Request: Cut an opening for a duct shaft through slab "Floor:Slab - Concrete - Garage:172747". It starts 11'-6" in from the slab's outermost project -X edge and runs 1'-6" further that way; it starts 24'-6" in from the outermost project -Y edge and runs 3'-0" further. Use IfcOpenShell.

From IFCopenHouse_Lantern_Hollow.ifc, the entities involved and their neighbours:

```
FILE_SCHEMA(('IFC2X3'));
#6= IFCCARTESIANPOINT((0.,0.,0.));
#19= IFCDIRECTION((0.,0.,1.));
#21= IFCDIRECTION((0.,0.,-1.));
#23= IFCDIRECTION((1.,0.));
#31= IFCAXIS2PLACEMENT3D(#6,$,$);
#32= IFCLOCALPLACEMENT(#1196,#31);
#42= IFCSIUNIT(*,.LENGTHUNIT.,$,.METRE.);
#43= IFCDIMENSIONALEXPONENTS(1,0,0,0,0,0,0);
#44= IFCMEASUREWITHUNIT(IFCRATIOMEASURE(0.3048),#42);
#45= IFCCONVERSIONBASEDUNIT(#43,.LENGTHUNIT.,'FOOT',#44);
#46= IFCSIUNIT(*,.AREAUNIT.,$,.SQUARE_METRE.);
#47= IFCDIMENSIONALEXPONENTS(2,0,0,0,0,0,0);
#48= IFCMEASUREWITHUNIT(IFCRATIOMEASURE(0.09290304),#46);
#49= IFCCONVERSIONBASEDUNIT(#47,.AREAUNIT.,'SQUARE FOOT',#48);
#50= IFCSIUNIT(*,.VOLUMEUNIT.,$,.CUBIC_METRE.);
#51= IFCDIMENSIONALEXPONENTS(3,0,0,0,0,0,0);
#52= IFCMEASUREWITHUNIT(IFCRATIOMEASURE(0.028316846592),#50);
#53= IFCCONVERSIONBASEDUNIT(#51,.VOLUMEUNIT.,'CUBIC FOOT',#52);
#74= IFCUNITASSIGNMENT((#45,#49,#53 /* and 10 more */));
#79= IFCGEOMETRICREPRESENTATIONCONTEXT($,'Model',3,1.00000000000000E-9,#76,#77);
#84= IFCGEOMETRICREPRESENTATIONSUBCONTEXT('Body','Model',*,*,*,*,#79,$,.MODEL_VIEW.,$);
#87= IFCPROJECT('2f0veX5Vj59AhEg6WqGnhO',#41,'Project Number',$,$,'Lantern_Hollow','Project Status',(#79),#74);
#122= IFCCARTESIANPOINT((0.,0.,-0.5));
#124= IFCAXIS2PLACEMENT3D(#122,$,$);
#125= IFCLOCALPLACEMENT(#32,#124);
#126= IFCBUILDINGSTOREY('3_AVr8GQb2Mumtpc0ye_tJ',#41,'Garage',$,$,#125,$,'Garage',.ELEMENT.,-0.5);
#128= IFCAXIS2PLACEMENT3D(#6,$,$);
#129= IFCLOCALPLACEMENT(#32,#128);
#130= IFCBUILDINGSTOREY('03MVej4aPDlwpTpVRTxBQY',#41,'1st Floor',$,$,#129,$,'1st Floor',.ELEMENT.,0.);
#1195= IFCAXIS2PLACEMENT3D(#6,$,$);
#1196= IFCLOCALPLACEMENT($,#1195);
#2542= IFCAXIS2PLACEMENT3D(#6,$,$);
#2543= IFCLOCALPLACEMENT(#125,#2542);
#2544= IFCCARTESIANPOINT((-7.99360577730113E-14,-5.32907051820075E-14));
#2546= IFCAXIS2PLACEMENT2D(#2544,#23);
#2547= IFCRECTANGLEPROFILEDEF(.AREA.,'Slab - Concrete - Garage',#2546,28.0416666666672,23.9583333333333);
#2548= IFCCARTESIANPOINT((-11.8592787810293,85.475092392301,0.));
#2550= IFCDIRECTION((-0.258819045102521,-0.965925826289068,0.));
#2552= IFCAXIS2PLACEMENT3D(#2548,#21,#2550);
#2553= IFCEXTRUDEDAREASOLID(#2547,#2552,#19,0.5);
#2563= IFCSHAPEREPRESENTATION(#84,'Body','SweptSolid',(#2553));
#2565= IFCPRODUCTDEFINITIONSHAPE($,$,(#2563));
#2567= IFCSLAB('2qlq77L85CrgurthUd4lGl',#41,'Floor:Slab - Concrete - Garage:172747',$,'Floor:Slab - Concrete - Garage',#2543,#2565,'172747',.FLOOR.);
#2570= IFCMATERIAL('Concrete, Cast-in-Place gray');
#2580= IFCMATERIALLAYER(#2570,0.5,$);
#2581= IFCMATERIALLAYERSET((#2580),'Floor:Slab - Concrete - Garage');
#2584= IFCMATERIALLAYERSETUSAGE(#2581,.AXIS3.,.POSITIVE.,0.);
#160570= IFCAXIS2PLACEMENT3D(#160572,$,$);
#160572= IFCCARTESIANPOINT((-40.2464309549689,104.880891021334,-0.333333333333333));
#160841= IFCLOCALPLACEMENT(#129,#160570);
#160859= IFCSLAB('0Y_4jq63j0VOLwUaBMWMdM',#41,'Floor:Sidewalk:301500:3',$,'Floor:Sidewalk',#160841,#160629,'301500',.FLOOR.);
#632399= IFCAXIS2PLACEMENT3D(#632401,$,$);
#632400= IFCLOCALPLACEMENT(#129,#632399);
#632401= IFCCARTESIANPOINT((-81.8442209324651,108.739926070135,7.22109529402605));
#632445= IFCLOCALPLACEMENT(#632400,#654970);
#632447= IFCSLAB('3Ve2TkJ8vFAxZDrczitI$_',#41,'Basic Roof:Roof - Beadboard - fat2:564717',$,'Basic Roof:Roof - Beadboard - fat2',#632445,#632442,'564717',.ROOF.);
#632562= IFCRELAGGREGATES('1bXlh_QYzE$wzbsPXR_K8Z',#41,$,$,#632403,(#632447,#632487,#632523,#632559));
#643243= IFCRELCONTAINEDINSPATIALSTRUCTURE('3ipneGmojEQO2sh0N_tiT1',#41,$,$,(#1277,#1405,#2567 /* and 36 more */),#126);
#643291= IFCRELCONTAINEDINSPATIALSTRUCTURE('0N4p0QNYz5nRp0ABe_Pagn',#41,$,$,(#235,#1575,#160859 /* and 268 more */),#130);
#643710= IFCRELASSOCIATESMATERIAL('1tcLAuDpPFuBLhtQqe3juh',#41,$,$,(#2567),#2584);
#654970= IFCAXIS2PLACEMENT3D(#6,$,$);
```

```python
import numpy as np
import ifcopenshell
import ifcopenshell.api.feature
import ifcopenshell.api.geometry
import ifcopenshell.api.root
import ifcopenshell.geom
import ifcopenshell.util.placement
import ifcopenshell.util.representation
import ifcopenshell.util.shape
import ifcopenshell.util.unit

model = ifcopenshell.open("IFCopenHouse_Lantern_Hollow.ifc")
unit_scale = ifcopenshell.util.unit.calculate_unit_scale(model)
settings = ifcopenshell.geom.settings()


def volume(element):
    """Net volume in cubic metres, openings subtracted."""
    shape = ifcopenshell.geom.create_shape(settings, element)
    return ifcopenshell.util.shape.get_volume(shape.geometry)


slab = model.by_id(2567)
before = volume(slab)

# Extent in the slab's own axes, in metres. The edges named are its -X and -Y sides.
slab_shape = ifcopenshell.geom.create_shape(settings, slab)
vertices = ifcopenshell.util.shape.get_vertices(slab_shape.geometry)
x_min, y_min, bottom = vertices.min(axis=0)
top = vertices[:, 2].max()

opening = ifcopenshell.api.root.create_entity(model, ifc_class="IfcOpeningElement", name="Duct shaft opening")
context = ifcopenshell.util.representation.get_context(model, "Model", "Body", "MODEL_VIEW")
width, depth = 0.4572, 0.9144
outline = [(0.0, 0.0), (width, 0.0), (width, depth), (0.0, depth), (0.0, 0.0)]
# Overshoot both faces by 50 mm so the cut is clean.
shape = ifcopenshell.api.geometry.add_slab_representation(
    model, context=context, depth=top - bottom + 0.1, polyline=outline
)
ifcopenshell.api.geometry.assign_representation(model, product=opening, representation=shape)

matrix = ifcopenshell.util.placement.get_local_placement(slab.ObjectPlacement)
matrix[:, 3] = matrix @ np.append(np.array([x_min + 3.5052, y_min + 7.4676, bottom - 0.05]) / unit_scale, 1.0)
ifcopenshell.api.geometry.edit_object_placement(model, product=opening, matrix=matrix, is_si=False)
ifcopenshell.api.feature.add_feature(model, feature=opening, element=slab)

after = volume(slab)

print(f"slab volume {before:.3f} -> {after:.3f} m3")

model.write("IFCopenHouse_Lantern_Hollow_rev.ifc")
```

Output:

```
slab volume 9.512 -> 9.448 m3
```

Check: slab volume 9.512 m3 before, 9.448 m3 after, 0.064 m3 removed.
